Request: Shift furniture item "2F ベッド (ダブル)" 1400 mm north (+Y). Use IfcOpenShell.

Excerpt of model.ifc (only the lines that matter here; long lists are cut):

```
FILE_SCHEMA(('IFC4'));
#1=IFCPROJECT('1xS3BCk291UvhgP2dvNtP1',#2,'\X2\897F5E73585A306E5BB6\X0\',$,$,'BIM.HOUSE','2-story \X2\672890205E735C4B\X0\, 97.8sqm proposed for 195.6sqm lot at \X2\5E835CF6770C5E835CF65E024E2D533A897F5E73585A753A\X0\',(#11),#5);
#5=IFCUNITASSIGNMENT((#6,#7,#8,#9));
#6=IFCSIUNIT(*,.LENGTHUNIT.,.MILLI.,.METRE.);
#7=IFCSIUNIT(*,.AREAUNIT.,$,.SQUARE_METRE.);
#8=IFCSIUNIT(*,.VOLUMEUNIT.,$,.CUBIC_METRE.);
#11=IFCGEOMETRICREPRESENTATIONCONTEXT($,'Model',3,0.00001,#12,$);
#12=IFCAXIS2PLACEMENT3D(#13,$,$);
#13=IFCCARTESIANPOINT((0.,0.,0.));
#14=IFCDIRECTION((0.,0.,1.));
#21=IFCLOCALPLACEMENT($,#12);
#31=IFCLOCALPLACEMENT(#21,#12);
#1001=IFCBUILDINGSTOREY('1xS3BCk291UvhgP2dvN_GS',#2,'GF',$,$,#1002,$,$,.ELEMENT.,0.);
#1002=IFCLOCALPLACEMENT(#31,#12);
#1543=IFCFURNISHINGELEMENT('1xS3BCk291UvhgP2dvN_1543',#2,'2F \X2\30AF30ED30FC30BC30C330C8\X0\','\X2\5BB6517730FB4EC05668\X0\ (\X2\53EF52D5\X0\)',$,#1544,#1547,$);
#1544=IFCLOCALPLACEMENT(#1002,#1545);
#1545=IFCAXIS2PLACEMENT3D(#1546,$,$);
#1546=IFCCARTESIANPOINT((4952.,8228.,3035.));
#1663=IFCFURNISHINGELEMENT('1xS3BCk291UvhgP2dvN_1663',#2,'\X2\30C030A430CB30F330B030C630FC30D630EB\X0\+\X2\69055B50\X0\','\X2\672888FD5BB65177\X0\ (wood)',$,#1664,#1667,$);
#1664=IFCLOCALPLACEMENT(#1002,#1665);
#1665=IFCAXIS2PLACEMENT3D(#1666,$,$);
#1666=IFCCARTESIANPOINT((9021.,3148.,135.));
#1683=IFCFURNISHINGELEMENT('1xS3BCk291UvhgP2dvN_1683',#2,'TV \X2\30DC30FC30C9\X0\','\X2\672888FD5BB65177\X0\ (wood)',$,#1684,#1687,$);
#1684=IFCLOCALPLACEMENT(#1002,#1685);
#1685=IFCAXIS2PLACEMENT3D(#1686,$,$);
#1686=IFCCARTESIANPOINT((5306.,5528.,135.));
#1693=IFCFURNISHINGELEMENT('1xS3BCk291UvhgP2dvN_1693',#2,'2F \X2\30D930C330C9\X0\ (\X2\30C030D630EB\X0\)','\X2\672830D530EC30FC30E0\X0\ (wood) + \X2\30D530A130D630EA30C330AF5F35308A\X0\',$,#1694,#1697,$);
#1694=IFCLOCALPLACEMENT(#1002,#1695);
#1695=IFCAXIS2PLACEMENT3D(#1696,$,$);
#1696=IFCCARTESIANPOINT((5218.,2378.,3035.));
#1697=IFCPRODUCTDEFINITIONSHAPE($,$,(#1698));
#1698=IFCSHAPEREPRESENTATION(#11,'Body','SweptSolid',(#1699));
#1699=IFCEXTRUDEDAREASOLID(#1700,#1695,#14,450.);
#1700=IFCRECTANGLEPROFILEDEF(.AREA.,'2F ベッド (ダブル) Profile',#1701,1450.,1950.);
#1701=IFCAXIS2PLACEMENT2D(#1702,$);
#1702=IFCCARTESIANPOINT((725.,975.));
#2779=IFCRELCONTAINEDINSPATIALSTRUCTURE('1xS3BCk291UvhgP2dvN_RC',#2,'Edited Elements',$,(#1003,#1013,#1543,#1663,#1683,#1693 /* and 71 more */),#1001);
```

```python
import ifcopenshell
import ifcopenshell.api.geometry
import ifcopenshell.util.placement

model = ifcopenshell.open("model.ifc")

item = model.by_id(1693)
matrix = ifcopenshell.util.placement.get_local_placement(item.ObjectPlacement)
matrix[1, 3] += 1400.0
ifcopenshell.api.geometry.edit_object_placement(model, product=item, matrix=matrix, is_si=False)

print(ifcopenshell.util.placement.get_local_placement(item.ObjectPlacement).round(3) + 0.0)

model.write("model_updated.ifc")
```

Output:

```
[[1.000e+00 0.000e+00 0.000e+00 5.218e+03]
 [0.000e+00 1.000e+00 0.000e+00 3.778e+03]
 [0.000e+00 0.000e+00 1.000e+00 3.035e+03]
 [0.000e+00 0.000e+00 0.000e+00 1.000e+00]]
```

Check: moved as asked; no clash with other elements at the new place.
